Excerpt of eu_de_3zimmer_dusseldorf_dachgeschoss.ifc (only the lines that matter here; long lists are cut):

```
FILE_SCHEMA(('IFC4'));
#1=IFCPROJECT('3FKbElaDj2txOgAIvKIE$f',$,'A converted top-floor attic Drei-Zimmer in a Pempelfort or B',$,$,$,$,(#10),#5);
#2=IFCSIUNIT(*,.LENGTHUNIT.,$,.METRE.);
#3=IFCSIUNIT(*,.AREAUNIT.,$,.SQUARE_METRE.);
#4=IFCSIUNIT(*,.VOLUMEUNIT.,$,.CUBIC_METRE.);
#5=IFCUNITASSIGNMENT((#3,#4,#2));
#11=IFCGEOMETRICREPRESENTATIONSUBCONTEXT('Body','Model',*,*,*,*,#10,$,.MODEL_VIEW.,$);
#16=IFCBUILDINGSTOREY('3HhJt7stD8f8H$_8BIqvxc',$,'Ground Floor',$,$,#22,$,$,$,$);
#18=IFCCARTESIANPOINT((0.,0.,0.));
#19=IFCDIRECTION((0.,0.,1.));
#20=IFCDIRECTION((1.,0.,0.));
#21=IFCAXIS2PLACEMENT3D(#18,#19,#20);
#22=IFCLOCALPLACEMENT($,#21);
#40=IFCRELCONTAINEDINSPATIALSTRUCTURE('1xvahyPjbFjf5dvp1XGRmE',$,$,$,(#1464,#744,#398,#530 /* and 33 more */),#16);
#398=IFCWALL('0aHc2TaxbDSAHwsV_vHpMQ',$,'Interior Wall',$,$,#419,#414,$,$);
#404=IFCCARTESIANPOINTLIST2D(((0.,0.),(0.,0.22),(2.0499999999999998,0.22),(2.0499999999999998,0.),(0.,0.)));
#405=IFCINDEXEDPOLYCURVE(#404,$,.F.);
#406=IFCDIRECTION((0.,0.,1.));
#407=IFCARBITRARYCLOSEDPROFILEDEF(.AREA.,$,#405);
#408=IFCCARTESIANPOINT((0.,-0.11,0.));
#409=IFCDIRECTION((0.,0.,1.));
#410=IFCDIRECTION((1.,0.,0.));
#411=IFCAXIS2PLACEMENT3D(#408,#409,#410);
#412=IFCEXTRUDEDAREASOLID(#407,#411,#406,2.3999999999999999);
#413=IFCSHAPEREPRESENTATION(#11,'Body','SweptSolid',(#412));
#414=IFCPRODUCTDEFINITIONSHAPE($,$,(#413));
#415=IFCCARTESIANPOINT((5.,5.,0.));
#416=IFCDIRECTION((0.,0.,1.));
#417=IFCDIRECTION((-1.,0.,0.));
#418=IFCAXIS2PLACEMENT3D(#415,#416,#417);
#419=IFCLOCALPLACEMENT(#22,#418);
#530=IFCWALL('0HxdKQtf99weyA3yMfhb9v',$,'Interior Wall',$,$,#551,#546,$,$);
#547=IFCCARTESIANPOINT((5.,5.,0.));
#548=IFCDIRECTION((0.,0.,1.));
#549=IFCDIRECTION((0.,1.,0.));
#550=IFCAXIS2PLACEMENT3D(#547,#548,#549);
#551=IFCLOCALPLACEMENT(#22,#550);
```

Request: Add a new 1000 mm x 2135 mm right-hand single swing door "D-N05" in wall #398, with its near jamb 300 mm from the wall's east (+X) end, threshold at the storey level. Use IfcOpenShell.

```python
import numpy as np
import ifcopenshell
import ifcopenshell.api.feature
import ifcopenshell.api.geometry
import ifcopenshell.api.root
import ifcopenshell.api.spatial
import ifcopenshell.geom
import ifcopenshell.util.element
import ifcopenshell.util.placement
import ifcopenshell.util.representation
import ifcopenshell.util.shape
import ifcopenshell.util.unit

model = ifcopenshell.open("eu_de_3zimmer_dusseldorf_dachgeschoss.ifc")
unit_scale = ifcopenshell.util.unit.calculate_unit_scale(model)
settings = ifcopenshell.geom.settings()


def volume(element):
    """Net volume in cubic metres, openings subtracted."""
    shape = ifcopenshell.geom.create_shape(settings, element)
    return ifcopenshell.util.shape.get_volume(shape.geometry)


wall = model.by_id(398)
storey = ifcopenshell.util.element.get_container(wall, ifc_class="IfcBuildingStorey")
context = ifcopenshell.util.representation.get_context(model, "Model", "Body", "MODEL_VIEW")
before = volume(wall)

width, height, from_end, sill = 1, 2.135, 0.3, 0.0  # metres

# The wall runs along its own X axis, and the end named is its -X end.
wall_shape = ifcopenshell.geom.create_shape(settings, wall)
x, y, z = ifcopenshell.util.shape.get_vertices(wall_shape.geometry).T
start = x.min() + from_end
face, thickness = float(y.min()), float(y.max() - y.min())
wall_matrix = ifcopenshell.util.placement.get_local_placement(wall.ObjectPlacement)
level = ifcopenshell.util.placement.get_local_placement(storey.ObjectPlacement)[2, 3]


def in_wall(x, y):
    """Placement at x, y metres in the wall's axes, at sill height."""
    matrix = wall_matrix.copy()
    matrix[:, 3] = wall_matrix @ np.array([x / unit_scale, y / unit_scale, 0.0, 1.0])
    matrix[2, 3] = level + sill / unit_scale
    return matrix


# Opening: a box that overshoots both wall faces by 50 mm.
opening = ifcopenshell.api.root.create_entity(model, ifc_class="IfcOpeningElement", predefined_type="OPENING")
box = ifcopenshell.api.geometry.add_wall_representation(
    model, context=context, length=width, height=height, thickness=thickness + 0.1
)
ifcopenshell.api.geometry.assign_representation(model, product=opening, representation=box)
ifcopenshell.api.geometry.edit_object_placement(model, product=opening, matrix=in_wall(start, face - 0.05), is_si=False)
ifcopenshell.api.feature.add_feature(model, feature=opening, element=wall)

door = ifcopenshell.api.root.create_entity(model, ifc_class="IfcDoor", name="D-N05", predefined_type="DOOR")
door.OverallWidth, door.OverallHeight = width / unit_scale, height / unit_scale
door.OperationType = "SINGLE_SWING_RIGHT"
body = ifcopenshell.api.geometry.add_door_representation(
    model,
    context=context,
    overall_width=door.OverallWidth,
    overall_height=door.OverallHeight,
    operation_type="SINGLE_SWING_RIGHT",
    lining_properties={"LiningDepth": thickness / unit_scale, "ThresholdDepth": thickness / unit_scale},
)
ifcopenshell.api.geometry.assign_representation(model, product=door, representation=body)
ifcopenshell.api.spatial.assign_container(model, products=[door], relating_structure=storey)
ifcopenshell.api.feature.add_filling(model, opening=opening, element=door)

# The lining spans the wall, so the door starts at the wall face.
ifcopenshell.api.geometry.edit_object_placement(model, product=door, matrix=in_wall(start, face), is_si=False)

after = volume(wall)

print(f"wall volume {before:.3f} -> {after:.3f} m3")

model.write("eu_de_3zimmer_dusseldorf_dachgeschoss_v2.ifc")
```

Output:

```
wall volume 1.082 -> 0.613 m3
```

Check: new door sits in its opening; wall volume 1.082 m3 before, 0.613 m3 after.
